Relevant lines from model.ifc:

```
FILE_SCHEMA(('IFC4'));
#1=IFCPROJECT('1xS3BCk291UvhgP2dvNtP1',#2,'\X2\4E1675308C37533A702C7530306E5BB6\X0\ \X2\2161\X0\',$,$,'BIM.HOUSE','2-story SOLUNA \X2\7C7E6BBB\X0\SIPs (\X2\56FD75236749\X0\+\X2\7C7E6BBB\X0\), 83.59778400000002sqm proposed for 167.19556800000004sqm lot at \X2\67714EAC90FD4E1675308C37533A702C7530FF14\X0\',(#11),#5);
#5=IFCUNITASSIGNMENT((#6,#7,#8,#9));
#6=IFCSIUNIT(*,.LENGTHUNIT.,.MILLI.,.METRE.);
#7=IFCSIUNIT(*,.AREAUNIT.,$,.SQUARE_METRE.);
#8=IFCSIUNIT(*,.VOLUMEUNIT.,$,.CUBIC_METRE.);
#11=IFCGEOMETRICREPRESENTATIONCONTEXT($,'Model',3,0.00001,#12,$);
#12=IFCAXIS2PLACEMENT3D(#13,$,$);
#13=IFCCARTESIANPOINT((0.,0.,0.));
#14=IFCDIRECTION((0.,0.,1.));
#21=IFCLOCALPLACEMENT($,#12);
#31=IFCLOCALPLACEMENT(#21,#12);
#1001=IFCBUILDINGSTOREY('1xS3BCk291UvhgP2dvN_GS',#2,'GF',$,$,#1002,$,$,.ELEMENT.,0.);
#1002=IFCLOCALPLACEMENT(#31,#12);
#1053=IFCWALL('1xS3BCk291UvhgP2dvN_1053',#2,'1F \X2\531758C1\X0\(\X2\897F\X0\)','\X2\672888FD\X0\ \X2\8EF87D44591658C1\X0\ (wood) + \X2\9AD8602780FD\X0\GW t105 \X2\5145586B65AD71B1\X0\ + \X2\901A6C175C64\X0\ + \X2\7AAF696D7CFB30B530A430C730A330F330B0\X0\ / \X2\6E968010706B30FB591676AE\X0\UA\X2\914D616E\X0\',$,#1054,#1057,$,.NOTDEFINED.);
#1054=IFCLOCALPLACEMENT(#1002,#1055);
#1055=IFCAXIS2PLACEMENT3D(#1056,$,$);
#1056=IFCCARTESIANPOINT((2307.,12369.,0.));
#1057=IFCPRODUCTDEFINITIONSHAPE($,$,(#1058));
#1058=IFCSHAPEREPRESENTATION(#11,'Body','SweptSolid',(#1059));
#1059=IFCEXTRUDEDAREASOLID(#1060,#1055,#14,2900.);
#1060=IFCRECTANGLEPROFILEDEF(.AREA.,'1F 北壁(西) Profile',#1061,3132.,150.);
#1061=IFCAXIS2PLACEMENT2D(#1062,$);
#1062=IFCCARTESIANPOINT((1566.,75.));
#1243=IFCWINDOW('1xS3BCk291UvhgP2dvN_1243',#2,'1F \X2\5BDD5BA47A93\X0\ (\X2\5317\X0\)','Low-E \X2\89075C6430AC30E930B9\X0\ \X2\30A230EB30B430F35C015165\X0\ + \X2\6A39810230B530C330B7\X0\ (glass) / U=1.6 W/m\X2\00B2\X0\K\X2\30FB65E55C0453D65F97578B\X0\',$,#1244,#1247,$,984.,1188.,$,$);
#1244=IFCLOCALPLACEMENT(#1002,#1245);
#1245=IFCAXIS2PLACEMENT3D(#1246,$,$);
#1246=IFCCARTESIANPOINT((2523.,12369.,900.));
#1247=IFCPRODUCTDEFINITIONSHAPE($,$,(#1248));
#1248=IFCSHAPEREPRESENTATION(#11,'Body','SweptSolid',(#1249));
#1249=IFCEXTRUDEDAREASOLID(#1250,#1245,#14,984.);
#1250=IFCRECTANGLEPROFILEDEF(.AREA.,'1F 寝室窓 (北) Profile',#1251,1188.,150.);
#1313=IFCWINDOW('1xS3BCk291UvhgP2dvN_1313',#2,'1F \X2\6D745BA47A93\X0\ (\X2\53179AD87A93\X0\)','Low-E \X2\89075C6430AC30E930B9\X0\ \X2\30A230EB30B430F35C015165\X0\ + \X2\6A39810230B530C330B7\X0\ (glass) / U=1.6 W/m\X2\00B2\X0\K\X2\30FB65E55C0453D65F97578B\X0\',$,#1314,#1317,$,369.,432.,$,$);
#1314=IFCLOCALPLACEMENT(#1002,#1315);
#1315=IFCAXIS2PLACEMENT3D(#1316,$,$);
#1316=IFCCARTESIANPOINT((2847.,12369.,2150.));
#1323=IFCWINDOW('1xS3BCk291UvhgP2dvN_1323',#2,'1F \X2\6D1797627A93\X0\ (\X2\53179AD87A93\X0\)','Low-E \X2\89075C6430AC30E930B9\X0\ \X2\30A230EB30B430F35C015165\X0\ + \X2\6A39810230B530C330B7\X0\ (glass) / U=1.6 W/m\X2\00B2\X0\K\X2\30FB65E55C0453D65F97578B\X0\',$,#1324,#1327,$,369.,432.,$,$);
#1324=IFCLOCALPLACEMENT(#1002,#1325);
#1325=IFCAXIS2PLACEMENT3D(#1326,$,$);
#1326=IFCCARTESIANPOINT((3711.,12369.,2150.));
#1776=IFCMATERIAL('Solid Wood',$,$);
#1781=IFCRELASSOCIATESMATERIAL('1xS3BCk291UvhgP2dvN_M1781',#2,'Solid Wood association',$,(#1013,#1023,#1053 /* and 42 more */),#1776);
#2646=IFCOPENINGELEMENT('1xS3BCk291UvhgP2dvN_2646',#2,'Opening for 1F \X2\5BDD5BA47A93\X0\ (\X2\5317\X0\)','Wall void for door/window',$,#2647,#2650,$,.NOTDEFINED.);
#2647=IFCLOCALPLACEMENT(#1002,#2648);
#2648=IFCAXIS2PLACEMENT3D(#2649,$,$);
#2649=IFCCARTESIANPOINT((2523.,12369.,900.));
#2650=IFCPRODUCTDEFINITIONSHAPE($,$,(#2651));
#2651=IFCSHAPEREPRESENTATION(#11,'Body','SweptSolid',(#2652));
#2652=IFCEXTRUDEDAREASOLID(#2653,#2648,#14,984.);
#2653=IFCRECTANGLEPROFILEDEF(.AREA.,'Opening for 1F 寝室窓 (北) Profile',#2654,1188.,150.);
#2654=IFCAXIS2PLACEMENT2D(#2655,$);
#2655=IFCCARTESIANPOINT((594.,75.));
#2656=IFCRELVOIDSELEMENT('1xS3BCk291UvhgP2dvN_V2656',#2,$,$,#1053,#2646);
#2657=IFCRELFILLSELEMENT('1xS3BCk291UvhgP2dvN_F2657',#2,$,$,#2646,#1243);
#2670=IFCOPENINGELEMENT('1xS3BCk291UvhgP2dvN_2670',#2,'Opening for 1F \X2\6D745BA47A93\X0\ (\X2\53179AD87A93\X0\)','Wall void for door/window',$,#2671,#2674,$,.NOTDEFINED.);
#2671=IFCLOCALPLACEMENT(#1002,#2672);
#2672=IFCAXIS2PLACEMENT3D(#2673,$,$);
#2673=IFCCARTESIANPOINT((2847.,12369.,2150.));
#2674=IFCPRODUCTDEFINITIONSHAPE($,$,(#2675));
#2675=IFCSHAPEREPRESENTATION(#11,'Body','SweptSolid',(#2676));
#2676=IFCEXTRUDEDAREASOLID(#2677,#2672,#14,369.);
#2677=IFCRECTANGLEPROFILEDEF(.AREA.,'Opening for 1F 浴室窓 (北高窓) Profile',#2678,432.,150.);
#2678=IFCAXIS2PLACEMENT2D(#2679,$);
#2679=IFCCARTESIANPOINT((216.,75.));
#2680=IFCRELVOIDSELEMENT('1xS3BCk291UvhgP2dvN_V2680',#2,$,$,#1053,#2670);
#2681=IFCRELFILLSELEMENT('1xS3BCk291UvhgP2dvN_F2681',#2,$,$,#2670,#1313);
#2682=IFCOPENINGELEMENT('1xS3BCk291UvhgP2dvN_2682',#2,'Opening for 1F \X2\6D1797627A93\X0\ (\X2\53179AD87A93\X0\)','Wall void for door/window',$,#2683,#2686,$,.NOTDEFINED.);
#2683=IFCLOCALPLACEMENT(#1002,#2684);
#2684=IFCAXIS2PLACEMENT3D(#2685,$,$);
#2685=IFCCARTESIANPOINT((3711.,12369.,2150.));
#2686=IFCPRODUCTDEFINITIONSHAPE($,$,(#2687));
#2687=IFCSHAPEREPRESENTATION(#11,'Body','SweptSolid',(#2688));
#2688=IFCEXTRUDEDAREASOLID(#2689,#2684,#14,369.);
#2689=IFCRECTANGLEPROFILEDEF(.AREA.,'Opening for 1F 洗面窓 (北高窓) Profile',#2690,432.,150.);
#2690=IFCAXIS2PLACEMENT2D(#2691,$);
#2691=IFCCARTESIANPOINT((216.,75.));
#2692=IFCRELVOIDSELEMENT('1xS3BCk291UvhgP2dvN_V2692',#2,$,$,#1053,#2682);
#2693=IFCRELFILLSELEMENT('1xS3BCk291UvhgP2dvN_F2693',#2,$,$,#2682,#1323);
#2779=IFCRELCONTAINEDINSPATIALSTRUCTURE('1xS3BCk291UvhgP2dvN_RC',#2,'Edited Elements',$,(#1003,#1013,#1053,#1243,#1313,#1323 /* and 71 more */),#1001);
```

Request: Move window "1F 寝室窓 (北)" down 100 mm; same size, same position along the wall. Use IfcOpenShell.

```python
import numpy as np
import ifcopenshell
import ifcopenshell.api.geometry
import ifcopenshell.util.placement
import ifcopenshell.util.unit

model = ifcopenshell.open("model.ifc")
unit_scale = ifcopenshell.util.unit.calculate_unit_scale(model)

window = model.by_guid("1xS3BCk291UvhgP2dvN_1243")
opening = window.FillsVoids[0].RelatingOpeningElement
dz = -0.1 / unit_scale

shift = np.array([0.0, 0.0, dz])
# The window is not placed relative to its opening, so move both.
for product in (opening, window):
    matrix = ifcopenshell.util.placement.get_local_placement(product.ObjectPlacement)
    matrix[:3, 3] += shift
    ifcopenshell.api.geometry.edit_object_placement(model, product=product, matrix=matrix, is_si=False)

print(f"moved by {dz * unit_scale:+.3f} m")

model.write("model_updated.ifc")
```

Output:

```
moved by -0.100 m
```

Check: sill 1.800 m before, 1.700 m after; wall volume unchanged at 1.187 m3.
